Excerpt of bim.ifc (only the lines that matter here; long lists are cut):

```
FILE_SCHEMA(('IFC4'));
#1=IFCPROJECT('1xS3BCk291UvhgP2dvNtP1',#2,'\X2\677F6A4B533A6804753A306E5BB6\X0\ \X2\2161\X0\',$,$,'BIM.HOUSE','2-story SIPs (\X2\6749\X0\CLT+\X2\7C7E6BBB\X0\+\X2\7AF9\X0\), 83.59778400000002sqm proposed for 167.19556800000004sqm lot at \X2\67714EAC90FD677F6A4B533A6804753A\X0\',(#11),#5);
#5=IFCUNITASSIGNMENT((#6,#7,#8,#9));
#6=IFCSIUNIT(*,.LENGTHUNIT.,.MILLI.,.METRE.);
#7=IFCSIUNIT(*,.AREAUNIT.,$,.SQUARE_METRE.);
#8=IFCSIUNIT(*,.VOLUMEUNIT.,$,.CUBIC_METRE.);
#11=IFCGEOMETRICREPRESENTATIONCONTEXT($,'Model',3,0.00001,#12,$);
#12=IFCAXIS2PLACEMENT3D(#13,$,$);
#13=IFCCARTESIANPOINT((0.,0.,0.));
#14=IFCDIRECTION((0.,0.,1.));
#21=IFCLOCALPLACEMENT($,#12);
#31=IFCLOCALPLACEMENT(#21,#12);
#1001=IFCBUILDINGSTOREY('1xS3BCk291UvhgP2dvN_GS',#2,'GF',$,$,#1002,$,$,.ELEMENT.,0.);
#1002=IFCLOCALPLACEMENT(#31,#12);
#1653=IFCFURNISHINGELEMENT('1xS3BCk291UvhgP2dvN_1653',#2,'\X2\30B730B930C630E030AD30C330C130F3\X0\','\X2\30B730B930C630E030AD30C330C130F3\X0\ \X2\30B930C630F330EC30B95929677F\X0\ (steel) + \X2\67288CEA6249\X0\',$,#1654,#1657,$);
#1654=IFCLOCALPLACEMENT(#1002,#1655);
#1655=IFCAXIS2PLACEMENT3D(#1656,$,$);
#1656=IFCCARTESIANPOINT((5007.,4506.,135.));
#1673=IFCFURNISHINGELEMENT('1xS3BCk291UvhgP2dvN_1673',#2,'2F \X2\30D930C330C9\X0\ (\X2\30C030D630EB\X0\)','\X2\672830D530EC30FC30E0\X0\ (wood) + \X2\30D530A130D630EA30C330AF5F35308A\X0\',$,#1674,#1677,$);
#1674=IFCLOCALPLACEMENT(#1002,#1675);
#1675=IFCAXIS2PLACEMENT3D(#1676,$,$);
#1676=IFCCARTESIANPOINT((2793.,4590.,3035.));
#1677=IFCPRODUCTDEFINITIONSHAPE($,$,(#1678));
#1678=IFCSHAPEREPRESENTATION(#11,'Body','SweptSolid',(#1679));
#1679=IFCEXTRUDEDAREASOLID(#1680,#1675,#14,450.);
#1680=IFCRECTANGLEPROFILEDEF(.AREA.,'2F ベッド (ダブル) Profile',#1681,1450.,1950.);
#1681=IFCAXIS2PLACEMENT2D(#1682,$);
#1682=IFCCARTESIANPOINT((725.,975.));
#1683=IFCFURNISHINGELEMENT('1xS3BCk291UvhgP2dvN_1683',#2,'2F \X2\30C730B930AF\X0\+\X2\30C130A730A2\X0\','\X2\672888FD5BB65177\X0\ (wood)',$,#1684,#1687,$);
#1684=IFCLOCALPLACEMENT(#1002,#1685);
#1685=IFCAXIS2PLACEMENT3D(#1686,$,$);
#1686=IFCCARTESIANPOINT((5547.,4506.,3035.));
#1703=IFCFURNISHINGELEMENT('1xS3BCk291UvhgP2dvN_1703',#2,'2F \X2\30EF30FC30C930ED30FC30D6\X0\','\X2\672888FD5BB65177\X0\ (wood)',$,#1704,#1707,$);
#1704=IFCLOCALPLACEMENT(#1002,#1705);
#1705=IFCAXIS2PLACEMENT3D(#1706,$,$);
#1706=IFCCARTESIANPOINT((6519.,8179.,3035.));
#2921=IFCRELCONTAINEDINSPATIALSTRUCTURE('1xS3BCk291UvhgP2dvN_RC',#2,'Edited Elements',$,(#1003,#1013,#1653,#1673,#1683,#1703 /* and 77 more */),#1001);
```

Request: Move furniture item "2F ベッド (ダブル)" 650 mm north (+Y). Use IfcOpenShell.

```python
import ifcopenshell
import ifcopenshell.api.geometry
import ifcopenshell.util.placement
import ifcopenshell.util.unit

model = ifcopenshell.open("bim.ifc")
unit_scale = ifcopenshell.util.unit.calculate_unit_scale(model)

item = model.by_guid("1xS3BCk291UvhgP2dvN_1673")
matrix = ifcopenshell.util.placement.get_local_placement(item.ObjectPlacement)
matrix[1, 3] += 0.65 / unit_scale
ifcopenshell.api.geometry.edit_object_placement(model, product=item, matrix=matrix, is_si=False)

print(ifcopenshell.util.placement.get_local_placement(item.ObjectPlacement).round(3) + 0.0)

model.write("bim_edited.ifc")
```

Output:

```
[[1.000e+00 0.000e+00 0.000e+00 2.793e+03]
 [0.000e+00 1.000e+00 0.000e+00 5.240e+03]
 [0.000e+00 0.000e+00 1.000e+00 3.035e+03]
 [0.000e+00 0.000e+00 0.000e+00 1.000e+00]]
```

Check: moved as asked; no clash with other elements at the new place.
